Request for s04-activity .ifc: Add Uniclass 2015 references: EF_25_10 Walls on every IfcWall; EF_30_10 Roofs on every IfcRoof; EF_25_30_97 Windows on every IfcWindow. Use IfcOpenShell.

First a look at what the model holds.

```python
import ifcopenshell

model = ifcopenshell.open("s04-activity .ifc")
print(model.schema)
print("classifications:", [c.Name for c in model.by_type("IfcClassification")])
for ifc_class in ("IfcDoor", "IfcRoof", "IfcStair", "IfcWall", "IfcWindow"):
    print(ifc_class, len(model.by_type(ifc_class)))
```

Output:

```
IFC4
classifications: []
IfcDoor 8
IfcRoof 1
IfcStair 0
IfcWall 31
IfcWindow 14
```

```python
import ifcopenshell
import ifcopenshell.api.classification

model = ifcopenshell.open("s04-activity .ifc")

system = ifcopenshell.api.classification.add_classification(model, classification="Uniclass 2015")

codes = {
    "IfcWall": ("EF_25_10", "Walls"),
    "IfcRoof": ("EF_30_10", "Roofs"),
    "IfcWindow": ("EF_25_30_97", "Windows"),
}
for ifc_class, (code, name) in codes.items():
    products = model.by_type(ifc_class)
    ifcopenshell.api.classification.add_reference(
        model, products=products, classification=system, identification=code, name=name
    )
    print(code, len(products))

model.write("s04-activity _edited.ifc")
```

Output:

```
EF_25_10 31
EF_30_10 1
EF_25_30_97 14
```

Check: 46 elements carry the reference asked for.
